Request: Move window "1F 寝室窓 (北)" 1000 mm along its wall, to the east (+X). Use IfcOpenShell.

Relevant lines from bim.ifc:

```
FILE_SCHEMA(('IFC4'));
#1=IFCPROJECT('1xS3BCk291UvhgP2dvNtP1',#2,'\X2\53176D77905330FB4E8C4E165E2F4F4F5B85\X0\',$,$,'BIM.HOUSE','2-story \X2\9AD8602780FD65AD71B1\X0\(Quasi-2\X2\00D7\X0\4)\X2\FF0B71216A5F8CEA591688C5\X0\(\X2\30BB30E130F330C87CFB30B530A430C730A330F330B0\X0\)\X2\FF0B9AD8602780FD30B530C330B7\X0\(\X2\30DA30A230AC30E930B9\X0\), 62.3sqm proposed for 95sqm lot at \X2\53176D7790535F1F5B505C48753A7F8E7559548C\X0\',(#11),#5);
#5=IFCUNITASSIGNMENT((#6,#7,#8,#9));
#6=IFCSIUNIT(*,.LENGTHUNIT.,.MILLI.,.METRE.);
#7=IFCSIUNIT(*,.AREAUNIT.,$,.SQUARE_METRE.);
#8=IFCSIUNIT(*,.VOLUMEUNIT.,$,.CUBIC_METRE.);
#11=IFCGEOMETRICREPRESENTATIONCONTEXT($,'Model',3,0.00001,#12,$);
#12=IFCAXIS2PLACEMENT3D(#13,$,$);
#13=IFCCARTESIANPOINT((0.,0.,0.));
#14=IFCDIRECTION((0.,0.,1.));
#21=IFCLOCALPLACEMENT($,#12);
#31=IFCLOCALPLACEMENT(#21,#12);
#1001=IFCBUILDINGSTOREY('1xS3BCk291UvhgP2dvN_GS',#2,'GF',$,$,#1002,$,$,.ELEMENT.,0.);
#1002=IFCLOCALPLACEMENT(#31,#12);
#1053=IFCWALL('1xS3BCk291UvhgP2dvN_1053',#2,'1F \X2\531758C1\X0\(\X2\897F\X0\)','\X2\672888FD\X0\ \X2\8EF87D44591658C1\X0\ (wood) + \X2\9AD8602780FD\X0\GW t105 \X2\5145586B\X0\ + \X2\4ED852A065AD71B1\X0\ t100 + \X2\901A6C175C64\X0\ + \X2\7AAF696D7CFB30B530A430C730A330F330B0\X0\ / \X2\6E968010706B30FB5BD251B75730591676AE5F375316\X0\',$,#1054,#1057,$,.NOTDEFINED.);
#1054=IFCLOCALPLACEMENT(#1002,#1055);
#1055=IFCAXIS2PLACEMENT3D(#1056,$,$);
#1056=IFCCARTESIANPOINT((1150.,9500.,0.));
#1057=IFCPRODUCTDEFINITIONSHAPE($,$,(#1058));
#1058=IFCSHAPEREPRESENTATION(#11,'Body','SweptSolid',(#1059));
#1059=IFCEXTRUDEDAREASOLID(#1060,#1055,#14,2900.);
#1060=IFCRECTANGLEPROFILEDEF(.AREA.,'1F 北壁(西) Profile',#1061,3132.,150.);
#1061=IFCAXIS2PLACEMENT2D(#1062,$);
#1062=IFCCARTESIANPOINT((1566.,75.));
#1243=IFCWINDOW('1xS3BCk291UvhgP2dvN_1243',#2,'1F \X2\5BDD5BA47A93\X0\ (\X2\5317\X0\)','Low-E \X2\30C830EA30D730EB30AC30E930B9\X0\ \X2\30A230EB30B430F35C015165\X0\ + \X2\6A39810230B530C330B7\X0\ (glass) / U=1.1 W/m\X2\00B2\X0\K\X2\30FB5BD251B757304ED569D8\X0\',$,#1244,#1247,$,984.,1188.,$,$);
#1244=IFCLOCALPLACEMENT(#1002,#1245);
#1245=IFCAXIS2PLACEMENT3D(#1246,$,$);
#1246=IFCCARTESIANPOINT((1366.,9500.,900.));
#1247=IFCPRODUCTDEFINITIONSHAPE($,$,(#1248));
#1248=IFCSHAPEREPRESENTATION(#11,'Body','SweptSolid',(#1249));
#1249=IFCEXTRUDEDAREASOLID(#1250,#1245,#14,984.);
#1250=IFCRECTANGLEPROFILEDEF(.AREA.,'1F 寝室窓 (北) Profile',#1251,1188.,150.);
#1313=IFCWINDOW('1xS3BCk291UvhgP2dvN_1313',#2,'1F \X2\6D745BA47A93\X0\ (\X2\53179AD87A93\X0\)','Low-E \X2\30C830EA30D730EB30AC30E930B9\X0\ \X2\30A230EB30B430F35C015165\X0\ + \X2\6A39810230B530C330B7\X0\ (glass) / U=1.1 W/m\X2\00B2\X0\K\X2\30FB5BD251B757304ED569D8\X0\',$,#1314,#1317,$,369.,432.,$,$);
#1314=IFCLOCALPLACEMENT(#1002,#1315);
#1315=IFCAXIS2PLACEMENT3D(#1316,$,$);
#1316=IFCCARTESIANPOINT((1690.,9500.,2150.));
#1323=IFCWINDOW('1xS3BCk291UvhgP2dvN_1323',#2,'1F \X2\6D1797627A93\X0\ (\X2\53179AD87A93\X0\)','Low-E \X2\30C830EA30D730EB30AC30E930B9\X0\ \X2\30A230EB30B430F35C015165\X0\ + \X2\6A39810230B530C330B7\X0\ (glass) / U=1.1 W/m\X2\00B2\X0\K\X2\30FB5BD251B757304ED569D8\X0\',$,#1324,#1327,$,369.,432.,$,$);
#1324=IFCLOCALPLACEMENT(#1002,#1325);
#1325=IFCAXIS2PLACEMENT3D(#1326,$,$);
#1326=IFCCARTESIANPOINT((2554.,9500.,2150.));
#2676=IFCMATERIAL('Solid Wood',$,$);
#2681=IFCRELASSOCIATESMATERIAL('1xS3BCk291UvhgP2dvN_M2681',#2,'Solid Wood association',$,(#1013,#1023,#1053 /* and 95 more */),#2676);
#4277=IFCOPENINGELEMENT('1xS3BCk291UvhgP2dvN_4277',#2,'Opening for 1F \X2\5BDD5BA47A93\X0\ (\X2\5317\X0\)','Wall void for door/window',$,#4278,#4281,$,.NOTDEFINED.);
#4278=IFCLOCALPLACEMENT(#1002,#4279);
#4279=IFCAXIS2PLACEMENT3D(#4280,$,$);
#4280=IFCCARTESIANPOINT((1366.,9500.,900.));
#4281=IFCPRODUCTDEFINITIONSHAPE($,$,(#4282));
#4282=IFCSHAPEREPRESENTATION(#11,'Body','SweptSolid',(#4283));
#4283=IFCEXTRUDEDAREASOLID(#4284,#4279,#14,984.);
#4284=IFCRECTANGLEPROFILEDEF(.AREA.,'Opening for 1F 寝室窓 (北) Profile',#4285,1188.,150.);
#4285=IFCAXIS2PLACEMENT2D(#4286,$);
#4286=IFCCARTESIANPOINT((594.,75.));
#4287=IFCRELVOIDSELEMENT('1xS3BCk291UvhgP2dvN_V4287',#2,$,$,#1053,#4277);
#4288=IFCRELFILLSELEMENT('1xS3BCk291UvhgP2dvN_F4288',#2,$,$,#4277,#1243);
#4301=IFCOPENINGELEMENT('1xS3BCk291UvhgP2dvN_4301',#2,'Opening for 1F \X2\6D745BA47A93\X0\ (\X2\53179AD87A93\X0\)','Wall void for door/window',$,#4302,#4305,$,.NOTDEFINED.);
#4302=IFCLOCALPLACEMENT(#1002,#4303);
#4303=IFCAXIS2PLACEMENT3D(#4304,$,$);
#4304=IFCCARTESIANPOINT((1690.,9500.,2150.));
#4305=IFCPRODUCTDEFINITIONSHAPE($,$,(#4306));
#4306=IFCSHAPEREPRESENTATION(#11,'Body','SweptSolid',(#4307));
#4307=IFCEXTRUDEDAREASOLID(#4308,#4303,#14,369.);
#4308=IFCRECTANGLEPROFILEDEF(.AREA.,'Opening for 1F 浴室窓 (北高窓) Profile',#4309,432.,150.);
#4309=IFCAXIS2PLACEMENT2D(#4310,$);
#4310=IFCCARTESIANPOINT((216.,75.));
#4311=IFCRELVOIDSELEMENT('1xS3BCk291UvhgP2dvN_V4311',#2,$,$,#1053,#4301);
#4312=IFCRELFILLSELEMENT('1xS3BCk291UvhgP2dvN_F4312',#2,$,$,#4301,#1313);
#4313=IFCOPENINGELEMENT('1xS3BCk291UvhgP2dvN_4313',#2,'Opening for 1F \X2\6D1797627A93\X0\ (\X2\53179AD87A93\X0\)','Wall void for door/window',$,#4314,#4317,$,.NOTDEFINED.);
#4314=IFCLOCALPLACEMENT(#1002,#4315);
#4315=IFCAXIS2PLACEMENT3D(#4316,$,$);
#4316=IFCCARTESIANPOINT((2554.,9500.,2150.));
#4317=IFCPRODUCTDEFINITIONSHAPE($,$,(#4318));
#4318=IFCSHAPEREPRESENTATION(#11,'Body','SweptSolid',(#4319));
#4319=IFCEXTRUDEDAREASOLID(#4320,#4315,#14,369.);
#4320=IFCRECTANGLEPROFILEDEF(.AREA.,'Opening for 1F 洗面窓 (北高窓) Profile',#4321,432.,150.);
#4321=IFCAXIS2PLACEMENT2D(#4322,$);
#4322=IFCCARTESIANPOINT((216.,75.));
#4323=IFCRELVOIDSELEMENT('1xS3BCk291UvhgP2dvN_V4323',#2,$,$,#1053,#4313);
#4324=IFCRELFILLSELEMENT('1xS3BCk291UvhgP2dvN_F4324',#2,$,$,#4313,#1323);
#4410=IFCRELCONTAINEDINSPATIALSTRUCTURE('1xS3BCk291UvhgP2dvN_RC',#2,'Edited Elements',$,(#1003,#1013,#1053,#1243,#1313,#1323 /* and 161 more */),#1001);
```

```python
import ifcopenshell
import ifcopenshell.api.geometry
import ifcopenshell.util.placement

model = ifcopenshell.open("bim.ifc")

window = model.by_guid("1xS3BCk291UvhgP2dvN_1243")
opening = window.FillsVoids[0].RelatingOpeningElement
wall = opening.VoidsElements[0].RelatingBuildingElement

wall_matrix = ifcopenshell.util.placement.get_local_placement(wall.ObjectPlacement)
shift = wall_matrix[:3, 0] * 1000.0
before = ifcopenshell.util.placement.get_local_placement(window.ObjectPlacement)[:3, 3].copy()

# The window is not placed relative to its opening, so move both.
for product in (opening, window):
    matrix = ifcopenshell.util.placement.get_local_placement(product.ObjectPlacement)
    matrix[:3, 3] += shift
    ifcopenshell.api.geometry.edit_object_placement(model, product=product, matrix=matrix, is_si=False)

after = ifcopenshell.util.placement.get_local_placement(window.ObjectPlacement)[:3, 3]
print("window moved by", (after - before).round(3) + 0.0)

model.write("bim_rev.ifc")
```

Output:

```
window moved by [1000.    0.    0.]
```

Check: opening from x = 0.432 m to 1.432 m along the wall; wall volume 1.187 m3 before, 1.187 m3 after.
